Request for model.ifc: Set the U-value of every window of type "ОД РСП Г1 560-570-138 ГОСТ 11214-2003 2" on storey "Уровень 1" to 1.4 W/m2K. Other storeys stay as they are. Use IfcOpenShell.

First a look at what the model holds.

```python
import ifcopenshell
import ifcopenshell.util.element

model = ifcopenshell.open("model.ifc")
print(model.schema)
storey = next(s for s in model.by_type("IfcBuildingStorey") if s.Name == "Уровень 1")
windows = [e for e in ifcopenshell.util.element.get_decomposition(storey) if e.is_a("IfcWindow")]
seen = {}
for e in windows:
    element_type = ifcopenshell.util.element.get_type(e)
    key = (element_type.Name if element_type != e and element_type else None, ifcopenshell.util.element.get_pset(e, "Pset_WindowCommon", "ThermalTransmittance"))
    seen[key] = seen.get(key, 0) + 1
for (name, value), count in sorted(seen.items(), key=str):
    print(count, "x", name, "|", value)
```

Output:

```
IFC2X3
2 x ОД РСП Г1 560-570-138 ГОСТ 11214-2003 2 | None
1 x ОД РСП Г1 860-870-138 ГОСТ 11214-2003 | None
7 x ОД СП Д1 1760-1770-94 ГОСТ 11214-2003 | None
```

```python
import ifcopenshell
import ifcopenshell.api.pset
import ifcopenshell.util.element

model = ifcopenshell.open("model.ifc")

storey = next(s for s in model.by_type("IfcBuildingStorey") if s.Name == "Уровень 1")
windows = [e for e in ifcopenshell.util.element.get_decomposition(storey) if e.is_a("IfcWindow")]

count = 0
for e in windows:
    element_type = ifcopenshell.util.element.get_type(e)
    if element_type in (None, e) or element_type.Name != "ОД РСП Г1 560-570-138 ГОСТ 11214-2003 2":
        continue
    # add_pset returns the element's existing set when there is one.
    pset = ifcopenshell.api.pset.add_pset(model, product=e, name="Pset_WindowCommon")
    ifcopenshell.api.pset.edit_pset(model, pset=pset, properties={"ThermalTransmittance": 1.4})
    count += 1

print(count, "windows updated")

model.write("model_edited.ifc")
```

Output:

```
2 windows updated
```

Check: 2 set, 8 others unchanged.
